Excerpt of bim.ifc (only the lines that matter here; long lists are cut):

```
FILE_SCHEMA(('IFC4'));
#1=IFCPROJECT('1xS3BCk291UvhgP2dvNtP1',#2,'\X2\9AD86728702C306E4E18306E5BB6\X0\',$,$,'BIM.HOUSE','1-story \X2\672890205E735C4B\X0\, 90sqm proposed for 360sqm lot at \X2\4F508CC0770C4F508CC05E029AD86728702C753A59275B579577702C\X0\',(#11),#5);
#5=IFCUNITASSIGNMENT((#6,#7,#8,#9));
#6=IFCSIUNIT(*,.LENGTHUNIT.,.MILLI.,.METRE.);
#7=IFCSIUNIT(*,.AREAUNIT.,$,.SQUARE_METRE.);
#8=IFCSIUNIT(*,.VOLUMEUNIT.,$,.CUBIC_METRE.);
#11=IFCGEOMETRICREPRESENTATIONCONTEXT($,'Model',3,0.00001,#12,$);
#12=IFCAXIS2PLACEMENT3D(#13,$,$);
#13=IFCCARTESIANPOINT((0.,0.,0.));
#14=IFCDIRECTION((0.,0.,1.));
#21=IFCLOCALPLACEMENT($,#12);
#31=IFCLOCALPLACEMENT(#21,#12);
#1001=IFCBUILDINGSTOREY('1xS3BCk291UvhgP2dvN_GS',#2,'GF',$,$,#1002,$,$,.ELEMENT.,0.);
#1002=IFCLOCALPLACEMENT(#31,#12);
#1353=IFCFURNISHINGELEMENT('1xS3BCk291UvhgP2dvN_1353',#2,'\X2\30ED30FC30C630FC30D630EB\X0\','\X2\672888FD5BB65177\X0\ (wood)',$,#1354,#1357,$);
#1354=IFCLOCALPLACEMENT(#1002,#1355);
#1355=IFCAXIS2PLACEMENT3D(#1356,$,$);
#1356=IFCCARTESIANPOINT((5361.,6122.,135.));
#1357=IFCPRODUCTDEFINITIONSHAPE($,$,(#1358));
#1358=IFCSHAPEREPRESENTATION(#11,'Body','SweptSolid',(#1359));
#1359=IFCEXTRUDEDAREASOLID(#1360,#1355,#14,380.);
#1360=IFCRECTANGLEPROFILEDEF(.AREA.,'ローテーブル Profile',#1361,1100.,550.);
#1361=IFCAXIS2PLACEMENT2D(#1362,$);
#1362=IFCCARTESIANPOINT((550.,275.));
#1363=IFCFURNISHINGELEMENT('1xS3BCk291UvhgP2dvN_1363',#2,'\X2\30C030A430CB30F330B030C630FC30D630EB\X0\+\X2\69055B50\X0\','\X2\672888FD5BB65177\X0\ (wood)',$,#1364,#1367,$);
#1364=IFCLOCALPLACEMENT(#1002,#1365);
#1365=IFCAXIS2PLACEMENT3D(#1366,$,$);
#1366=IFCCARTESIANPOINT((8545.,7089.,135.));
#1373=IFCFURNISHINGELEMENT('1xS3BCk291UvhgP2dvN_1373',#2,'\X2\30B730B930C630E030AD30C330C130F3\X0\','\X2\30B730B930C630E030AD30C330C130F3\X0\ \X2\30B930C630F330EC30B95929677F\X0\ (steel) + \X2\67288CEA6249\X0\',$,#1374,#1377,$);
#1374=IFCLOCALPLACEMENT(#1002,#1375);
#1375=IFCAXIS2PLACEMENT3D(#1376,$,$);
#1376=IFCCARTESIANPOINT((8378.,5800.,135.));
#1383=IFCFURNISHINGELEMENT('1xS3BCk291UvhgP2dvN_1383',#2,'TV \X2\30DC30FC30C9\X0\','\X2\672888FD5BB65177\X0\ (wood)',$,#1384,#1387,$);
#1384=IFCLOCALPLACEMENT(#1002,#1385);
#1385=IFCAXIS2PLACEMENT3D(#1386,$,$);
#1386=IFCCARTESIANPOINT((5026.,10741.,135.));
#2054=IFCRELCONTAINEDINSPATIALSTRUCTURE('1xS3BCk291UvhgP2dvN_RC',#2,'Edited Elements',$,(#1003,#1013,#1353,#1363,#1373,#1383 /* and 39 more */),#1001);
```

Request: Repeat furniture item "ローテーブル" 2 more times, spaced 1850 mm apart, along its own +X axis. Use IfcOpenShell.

```python
import ifcopenshell
import ifcopenshell.api.geometry
import ifcopenshell.api.root
import ifcopenshell.util.element
import ifcopenshell.util.placement

model = ifcopenshell.open("bim.ifc")


def reuse_history(source, copy):
    """copy_class also copies each property set's owner history, people and application; keep the originals."""
    for rel in copy.IsDefinedBy:
        if rel.is_a("IfcRelDefinesByProperties") and (history := rel.RelatingPropertyDefinition.OwnerHistory):
            rel.RelatingPropertyDefinition.OwnerHistory = source.OwnerHistory
            ifcopenshell.util.element.remove_deep2(model, history)


source = model.by_guid("1xS3BCk291UvhgP2dvN_1353")
base = ifcopenshell.util.placement.get_local_placement(source.ObjectPlacement)
step = base[:3, 0] * 1850.0

for i in range(1, 3):
    copy = ifcopenshell.api.root.copy_class(model, product=source)
    copy.Representation = ifcopenshell.util.element.copy_deep(
        model, source.Representation, exclude=["IfcGeometricRepresentationContext", "IfcRepresentationMap"]
    )
    reuse_history(source, copy)
    matrix = base.copy()
    matrix[:3, 3] += i * step
    print("added at", matrix[:3, 3].round(3) + 0.0)
    ifcopenshell.api.geometry.edit_object_placement(model, product=copy, matrix=matrix, is_si=False)

model.write("bim_updated.ifc")
```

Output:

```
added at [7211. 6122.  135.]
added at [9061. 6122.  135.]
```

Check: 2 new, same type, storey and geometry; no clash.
